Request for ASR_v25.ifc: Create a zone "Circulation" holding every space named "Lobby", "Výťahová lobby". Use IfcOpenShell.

First a look at what the model holds.

```python
import ifcopenshell

model = ifcopenshell.open("ASR_v25.ifc")
print(model.schema)
seen = {}
for space in model.by_type("IfcSpace"):
    seen[space.LongName] = seen.get(space.LongName, 0) + 1
for name, count in sorted(seen.items(), key=str):
    print(count, "x", name)
print("zones:", [z.Name for z in model.by_type("IfcZone")][:20])
```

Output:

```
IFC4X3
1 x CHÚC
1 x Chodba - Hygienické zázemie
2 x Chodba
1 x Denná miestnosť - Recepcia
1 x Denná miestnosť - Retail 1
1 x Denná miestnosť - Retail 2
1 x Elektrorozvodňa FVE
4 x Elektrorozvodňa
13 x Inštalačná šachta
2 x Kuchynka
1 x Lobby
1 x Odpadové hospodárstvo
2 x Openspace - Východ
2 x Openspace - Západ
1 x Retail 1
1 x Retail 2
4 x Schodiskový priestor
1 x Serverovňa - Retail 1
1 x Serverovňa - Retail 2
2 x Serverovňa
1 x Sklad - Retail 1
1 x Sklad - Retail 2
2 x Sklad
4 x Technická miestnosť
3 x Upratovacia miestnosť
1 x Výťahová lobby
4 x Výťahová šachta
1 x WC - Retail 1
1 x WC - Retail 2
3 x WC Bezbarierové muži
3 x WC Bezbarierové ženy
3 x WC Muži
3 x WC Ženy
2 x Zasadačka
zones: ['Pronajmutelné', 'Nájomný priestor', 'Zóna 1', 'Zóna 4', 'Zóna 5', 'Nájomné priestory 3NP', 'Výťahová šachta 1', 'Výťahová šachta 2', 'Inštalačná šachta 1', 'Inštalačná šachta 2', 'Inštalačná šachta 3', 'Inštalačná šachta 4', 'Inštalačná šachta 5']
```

```python
import ifcopenshell
import ifcopenshell.api.group
import ifcopenshell.api.root

model = ifcopenshell.open("ASR_v25.ifc")

names = {"Lobby", "Výťahová lobby"}
spaces = [s for s in model.by_type("IfcSpace") if s.LongName in names]

zone = ifcopenshell.api.root.create_entity(model, ifc_class="IfcZone", name="Circulation")
ifcopenshell.api.group.assign_group(model, products=spaces, group=zone)
print(len(spaces), "spaces in", zone.Name)

model.write("ASR_v25_rev.ifc")
```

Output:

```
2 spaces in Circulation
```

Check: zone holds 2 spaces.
